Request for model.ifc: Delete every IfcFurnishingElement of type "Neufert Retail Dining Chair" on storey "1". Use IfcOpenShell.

First a look at what the model holds.

```python
import ifcopenshell
import ifcopenshell.util.element

model = ifcopenshell.open("model.ifc")
print(model.schema)
storey = next(s for s in model.by_type("IfcBuildingStorey") if s.Name == "1")
furniture = [e for e in ifcopenshell.util.element.get_decomposition(storey) if e.is_a("IfcFurnishingElement")]
seen = {}
for e in furniture:
    element_type = ifcopenshell.util.element.get_type(e)
    name = element_type.Name if element_type not in (None, e) else None
    seen[name] = seen.get(name, 0) + 1
for name, count in sorted(seen.items(), key=str):
    print(count, "x", name)
```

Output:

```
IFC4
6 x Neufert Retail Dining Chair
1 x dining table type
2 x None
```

```python
import ifcopenshell
import ifcopenshell.api.root
import ifcopenshell.util.element

model = ifcopenshell.open("model.ifc")

storey = next(s for s in model.by_type("IfcBuildingStorey") if s.Name == "1")
furniture = [e for e in ifcopenshell.util.element.get_decomposition(storey) if e.is_a("IfcFurnishingElement")]
targets = [e for e in furniture if (t := ifcopenshell.util.element.get_type(e)) not in (None, e) and t.Name == "Neufert Retail Dining Chair"]

for e in targets:
    ifcopenshell.api.root.remove_product(model, product=e)
print(len(targets), "removed")

model.write("model_v2.ifc")
```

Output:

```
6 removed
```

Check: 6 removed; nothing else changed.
